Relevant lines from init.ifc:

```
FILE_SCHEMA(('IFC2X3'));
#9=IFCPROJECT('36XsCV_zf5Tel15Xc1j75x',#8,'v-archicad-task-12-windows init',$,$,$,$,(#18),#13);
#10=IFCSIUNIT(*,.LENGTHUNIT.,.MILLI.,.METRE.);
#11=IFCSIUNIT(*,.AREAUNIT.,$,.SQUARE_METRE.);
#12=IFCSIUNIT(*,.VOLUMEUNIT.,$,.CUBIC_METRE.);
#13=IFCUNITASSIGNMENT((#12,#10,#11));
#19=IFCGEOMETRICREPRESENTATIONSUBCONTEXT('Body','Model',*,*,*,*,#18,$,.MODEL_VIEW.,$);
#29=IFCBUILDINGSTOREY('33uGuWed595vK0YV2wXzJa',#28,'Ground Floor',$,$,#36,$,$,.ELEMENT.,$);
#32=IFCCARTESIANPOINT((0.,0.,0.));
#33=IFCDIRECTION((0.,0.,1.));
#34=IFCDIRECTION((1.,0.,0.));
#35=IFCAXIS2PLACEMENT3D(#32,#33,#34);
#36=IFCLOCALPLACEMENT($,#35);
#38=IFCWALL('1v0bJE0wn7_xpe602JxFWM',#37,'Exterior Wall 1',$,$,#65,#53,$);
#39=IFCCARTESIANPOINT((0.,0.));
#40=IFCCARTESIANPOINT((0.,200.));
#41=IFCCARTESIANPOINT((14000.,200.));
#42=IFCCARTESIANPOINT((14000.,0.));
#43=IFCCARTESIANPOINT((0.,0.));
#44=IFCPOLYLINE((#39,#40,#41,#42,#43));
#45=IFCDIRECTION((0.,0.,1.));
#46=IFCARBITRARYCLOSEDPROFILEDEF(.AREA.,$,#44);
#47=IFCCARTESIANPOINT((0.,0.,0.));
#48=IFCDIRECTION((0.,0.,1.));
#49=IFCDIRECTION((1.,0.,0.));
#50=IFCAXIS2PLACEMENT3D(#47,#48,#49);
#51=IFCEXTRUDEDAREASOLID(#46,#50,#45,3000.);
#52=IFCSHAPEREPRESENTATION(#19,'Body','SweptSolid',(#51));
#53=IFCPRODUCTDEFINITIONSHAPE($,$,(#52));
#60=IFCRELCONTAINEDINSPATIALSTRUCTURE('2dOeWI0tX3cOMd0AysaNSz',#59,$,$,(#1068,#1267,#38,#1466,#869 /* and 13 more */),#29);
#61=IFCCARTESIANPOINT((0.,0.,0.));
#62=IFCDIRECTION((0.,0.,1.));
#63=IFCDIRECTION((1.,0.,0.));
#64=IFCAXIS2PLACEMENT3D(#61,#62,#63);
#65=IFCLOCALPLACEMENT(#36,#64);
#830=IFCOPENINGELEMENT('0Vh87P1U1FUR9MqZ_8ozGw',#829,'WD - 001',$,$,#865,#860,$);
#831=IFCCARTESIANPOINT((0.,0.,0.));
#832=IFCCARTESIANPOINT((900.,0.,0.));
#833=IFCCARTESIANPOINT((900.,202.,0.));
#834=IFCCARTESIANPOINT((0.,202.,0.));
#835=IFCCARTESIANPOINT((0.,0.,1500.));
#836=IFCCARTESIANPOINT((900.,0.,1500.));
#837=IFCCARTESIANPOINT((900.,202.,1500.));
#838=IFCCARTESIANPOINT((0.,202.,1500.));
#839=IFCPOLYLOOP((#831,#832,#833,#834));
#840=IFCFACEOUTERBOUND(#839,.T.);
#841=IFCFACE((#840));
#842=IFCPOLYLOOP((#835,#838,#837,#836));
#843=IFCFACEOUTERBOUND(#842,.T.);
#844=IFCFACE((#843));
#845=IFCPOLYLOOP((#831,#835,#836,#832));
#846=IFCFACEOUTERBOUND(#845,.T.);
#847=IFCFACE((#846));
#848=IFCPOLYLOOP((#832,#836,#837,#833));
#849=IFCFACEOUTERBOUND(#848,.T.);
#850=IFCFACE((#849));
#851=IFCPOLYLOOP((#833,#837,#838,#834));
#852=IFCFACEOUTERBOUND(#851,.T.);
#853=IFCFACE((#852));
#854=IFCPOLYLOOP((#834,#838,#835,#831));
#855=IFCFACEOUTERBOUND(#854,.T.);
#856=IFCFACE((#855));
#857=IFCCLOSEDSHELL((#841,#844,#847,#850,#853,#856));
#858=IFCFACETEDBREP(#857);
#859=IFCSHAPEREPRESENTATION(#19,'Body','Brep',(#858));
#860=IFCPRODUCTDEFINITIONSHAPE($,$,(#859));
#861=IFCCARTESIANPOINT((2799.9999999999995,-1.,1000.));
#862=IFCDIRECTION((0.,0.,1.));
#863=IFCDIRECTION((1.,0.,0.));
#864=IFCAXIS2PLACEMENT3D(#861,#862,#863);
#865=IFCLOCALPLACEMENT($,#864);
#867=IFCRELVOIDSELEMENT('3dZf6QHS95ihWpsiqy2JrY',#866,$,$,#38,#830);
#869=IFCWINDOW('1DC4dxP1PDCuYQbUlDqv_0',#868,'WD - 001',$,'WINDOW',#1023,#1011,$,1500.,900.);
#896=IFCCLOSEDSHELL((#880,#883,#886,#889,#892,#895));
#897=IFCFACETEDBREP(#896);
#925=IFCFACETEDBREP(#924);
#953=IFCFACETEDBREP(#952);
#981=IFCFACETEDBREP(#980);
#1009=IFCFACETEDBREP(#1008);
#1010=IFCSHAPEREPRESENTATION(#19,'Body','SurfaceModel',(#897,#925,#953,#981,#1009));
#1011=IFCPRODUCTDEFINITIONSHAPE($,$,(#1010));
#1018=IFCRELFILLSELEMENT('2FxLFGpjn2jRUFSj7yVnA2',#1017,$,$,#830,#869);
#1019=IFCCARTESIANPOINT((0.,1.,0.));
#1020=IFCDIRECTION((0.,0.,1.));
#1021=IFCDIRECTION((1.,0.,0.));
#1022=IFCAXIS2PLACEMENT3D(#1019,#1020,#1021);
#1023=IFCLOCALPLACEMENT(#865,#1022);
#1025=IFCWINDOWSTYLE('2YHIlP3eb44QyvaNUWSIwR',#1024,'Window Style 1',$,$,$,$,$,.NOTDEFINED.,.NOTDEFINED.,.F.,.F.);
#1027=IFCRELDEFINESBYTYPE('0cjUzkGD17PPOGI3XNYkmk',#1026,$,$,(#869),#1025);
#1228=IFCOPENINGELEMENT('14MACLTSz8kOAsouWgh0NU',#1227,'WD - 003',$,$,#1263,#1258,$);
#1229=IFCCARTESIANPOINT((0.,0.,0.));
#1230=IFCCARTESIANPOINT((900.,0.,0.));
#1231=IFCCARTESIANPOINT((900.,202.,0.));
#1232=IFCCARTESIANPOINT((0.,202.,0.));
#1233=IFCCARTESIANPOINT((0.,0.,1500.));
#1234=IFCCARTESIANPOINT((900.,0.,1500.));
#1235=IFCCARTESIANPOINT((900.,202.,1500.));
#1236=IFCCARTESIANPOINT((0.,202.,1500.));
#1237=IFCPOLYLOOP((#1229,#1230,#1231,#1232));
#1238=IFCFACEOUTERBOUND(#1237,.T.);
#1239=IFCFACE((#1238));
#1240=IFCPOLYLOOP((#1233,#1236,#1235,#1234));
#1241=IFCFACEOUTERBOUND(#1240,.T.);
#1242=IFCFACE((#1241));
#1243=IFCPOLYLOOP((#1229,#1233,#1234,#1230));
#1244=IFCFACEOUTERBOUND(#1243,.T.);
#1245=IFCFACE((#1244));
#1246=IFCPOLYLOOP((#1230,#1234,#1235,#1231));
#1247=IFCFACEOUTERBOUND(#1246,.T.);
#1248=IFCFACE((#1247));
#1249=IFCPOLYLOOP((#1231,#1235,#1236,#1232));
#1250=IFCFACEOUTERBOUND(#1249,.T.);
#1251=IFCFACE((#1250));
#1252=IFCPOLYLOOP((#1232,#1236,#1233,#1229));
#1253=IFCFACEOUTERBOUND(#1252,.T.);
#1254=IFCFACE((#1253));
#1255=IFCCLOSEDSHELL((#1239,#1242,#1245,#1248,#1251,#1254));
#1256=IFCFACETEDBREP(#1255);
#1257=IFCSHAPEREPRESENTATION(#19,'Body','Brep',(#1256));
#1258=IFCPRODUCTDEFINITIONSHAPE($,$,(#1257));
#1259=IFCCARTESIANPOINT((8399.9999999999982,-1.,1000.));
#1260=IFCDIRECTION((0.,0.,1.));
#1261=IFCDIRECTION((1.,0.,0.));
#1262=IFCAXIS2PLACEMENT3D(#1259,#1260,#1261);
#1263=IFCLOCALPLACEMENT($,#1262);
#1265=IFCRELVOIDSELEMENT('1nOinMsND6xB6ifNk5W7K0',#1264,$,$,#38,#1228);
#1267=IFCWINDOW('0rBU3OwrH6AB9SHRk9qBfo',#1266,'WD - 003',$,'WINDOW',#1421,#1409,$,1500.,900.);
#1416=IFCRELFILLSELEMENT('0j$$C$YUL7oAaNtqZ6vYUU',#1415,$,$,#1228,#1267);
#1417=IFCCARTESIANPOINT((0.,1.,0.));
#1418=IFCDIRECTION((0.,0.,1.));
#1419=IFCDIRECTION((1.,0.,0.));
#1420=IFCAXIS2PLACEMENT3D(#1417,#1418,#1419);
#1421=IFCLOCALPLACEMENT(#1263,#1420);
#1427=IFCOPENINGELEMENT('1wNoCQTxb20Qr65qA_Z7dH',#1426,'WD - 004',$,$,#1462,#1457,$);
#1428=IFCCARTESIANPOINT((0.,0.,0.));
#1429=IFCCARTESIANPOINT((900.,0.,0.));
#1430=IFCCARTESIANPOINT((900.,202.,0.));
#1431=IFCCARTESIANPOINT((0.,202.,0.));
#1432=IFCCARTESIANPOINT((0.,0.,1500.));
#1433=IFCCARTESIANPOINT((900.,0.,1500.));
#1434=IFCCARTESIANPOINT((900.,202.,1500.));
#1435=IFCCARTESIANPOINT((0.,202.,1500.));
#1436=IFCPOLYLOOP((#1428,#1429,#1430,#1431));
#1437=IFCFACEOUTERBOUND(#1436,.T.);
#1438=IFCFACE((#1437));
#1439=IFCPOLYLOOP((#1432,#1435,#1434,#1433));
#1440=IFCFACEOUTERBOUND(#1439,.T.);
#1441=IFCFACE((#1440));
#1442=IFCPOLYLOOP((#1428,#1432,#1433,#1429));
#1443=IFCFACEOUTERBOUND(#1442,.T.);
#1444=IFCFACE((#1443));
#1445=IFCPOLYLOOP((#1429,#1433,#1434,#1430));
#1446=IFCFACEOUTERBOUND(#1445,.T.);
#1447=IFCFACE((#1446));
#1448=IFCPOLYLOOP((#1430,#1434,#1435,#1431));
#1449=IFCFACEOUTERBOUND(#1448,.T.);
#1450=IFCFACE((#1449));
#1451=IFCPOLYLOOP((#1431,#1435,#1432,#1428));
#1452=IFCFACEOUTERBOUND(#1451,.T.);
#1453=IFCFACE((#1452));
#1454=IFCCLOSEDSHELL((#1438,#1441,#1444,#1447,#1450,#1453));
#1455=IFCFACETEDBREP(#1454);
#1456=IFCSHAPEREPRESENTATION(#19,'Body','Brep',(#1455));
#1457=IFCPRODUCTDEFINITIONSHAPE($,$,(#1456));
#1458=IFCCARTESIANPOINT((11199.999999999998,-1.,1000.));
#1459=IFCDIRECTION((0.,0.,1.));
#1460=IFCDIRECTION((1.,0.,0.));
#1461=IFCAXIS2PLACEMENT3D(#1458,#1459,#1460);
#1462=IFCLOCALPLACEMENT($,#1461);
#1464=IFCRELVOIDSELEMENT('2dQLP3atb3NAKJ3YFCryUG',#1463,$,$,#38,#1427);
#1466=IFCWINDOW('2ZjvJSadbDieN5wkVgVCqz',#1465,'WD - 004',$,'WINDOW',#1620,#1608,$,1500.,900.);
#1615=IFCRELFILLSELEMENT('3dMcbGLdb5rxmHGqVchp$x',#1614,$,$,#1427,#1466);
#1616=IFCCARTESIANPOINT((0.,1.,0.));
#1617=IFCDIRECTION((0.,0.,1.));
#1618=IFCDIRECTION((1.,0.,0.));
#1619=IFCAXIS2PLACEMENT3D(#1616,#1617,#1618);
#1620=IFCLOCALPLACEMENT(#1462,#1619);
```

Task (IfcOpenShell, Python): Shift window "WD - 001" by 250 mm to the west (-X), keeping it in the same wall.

```python
import ifcopenshell
import ifcopenshell.api.geometry
import ifcopenshell.util.placement
import ifcopenshell.util.unit

model = ifcopenshell.open("init.ifc")
unit_scale = ifcopenshell.util.unit.calculate_unit_scale(model)

window = model.by_id(869)
opening = window.FillsVoids[0].RelatingOpeningElement
wall = opening.VoidsElements[0].RelatingBuildingElement

wall_matrix = ifcopenshell.util.placement.get_local_placement(wall.ObjectPlacement)
shift = wall_matrix[:3, 0] * -0.25 / unit_scale
before = ifcopenshell.util.placement.get_local_placement(window.ObjectPlacement)[:3, 3].copy()

# The window is placed relative to its opening, so it follows when the opening moves.
matrix = ifcopenshell.util.placement.get_local_placement(opening.ObjectPlacement)
matrix[:3, 3] += shift
ifcopenshell.api.geometry.edit_object_placement(
    model, product=opening, matrix=matrix, is_si=False, should_transform_children=True
)

after = ifcopenshell.util.placement.get_local_placement(window.ObjectPlacement)[:3, 3]
print("window moved by", (after - before).round(3) + 0.0)

model.write("init_v2.ifc")
```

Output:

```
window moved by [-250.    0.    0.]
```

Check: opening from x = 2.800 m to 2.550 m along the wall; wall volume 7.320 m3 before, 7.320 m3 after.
